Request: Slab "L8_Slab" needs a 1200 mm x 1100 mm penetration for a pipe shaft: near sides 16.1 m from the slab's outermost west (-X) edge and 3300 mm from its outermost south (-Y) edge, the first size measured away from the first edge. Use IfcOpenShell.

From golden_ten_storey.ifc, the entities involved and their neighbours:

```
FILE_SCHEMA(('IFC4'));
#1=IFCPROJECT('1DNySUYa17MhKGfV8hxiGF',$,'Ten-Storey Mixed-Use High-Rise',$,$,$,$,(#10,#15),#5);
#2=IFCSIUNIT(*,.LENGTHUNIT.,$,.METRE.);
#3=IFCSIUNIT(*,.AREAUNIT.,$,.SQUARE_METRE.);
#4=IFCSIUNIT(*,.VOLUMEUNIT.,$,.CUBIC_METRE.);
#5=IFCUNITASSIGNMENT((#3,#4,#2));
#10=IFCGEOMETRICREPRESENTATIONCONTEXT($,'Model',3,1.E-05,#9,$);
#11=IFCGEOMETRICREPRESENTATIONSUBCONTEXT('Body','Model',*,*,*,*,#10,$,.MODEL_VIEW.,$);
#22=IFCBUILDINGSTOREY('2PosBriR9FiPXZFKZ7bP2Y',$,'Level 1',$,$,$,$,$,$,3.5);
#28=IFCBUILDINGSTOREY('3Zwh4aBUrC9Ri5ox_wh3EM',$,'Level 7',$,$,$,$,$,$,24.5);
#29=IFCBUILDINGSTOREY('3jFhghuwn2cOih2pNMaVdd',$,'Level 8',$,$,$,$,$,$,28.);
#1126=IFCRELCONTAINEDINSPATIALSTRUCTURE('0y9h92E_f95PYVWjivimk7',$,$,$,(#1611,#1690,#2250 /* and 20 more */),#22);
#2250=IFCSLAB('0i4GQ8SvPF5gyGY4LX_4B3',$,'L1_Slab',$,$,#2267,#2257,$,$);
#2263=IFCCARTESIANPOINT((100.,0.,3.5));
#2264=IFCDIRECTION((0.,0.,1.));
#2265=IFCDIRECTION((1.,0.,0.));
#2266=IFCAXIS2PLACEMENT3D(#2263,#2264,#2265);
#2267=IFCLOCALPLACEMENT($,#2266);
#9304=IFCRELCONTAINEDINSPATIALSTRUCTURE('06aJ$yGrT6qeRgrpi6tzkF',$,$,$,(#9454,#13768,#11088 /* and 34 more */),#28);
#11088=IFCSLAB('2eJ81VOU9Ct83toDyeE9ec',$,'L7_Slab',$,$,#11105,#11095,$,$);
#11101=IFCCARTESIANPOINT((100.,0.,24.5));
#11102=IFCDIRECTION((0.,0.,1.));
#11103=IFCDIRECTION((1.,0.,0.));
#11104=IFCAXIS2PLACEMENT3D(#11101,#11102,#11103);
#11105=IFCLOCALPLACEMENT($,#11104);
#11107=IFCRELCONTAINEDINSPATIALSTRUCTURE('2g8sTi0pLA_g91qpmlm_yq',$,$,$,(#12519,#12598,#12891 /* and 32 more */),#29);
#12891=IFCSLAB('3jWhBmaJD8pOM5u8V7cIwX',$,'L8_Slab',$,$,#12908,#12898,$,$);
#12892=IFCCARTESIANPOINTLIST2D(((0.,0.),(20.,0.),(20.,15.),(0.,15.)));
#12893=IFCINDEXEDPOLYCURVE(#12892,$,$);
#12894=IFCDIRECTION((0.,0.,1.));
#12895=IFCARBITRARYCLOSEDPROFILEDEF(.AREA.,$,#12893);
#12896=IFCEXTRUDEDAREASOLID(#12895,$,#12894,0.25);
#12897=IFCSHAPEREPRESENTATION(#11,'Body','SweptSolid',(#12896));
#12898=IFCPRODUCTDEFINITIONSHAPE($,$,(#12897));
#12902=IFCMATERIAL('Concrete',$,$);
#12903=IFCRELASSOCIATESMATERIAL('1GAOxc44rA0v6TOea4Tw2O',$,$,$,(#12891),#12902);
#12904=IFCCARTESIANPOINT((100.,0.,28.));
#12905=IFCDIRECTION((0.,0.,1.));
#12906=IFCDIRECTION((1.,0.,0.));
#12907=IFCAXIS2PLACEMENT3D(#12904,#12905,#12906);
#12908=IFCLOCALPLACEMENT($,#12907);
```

```python
import numpy as np
import ifcopenshell
import ifcopenshell.api.feature
import ifcopenshell.api.geometry
import ifcopenshell.api.root
import ifcopenshell.geom
import ifcopenshell.util.placement
import ifcopenshell.util.representation
import ifcopenshell.util.shape
import ifcopenshell.util.unit

model = ifcopenshell.open("golden_ten_storey.ifc")
unit_scale = ifcopenshell.util.unit.calculate_unit_scale(model)
settings = ifcopenshell.geom.settings()


def volume(element):
    """Net volume in cubic metres, openings subtracted."""
    shape = ifcopenshell.geom.create_shape(settings, element)
    return ifcopenshell.util.shape.get_volume(shape.geometry)


slab = model.by_guid("3jWhBmaJD8pOM5u8V7cIwX")
before = volume(slab)

# Extent in the slab's own axes, in metres. The edges named are its -X and -Y sides.
slab_shape = ifcopenshell.geom.create_shape(settings, slab)
vertices = ifcopenshell.util.shape.get_vertices(slab_shape.geometry)
x_min, y_min, bottom = vertices.min(axis=0)
top = vertices[:, 2].max()

opening = ifcopenshell.api.root.create_entity(model, ifc_class="IfcOpeningElement", name="Pipe shaft opening", predefined_type="OPENING")
context = ifcopenshell.util.representation.get_context(model, "Model", "Body", "MODEL_VIEW")
width, depth = 1.2, 1.1
outline = [(0.0, 0.0), (width, 0.0), (width, depth), (0.0, depth), (0.0, 0.0)]
# Overshoot both faces by 50 mm so the cut is clean.
shape = ifcopenshell.api.geometry.add_slab_representation(
    model, context=context, depth=top - bottom + 0.1, polyline=outline
)
ifcopenshell.api.geometry.assign_representation(model, product=opening, representation=shape)

matrix = ifcopenshell.util.placement.get_local_placement(slab.ObjectPlacement)
matrix[:, 3] = matrix @ np.append(np.array([x_min + 16.1, y_min + 3.3, bottom - 0.05]) / unit_scale, 1.0)
ifcopenshell.api.geometry.edit_object_placement(model, product=opening, matrix=matrix, is_si=False)
ifcopenshell.api.feature.add_feature(model, feature=opening, element=slab)

after = volume(slab)

print(f"slab volume {before:.3f} -> {after:.3f} m3")

model.write("golden_ten_storey_v2.ifc")
```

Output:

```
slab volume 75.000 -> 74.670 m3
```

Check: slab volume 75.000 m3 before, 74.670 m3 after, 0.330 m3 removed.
